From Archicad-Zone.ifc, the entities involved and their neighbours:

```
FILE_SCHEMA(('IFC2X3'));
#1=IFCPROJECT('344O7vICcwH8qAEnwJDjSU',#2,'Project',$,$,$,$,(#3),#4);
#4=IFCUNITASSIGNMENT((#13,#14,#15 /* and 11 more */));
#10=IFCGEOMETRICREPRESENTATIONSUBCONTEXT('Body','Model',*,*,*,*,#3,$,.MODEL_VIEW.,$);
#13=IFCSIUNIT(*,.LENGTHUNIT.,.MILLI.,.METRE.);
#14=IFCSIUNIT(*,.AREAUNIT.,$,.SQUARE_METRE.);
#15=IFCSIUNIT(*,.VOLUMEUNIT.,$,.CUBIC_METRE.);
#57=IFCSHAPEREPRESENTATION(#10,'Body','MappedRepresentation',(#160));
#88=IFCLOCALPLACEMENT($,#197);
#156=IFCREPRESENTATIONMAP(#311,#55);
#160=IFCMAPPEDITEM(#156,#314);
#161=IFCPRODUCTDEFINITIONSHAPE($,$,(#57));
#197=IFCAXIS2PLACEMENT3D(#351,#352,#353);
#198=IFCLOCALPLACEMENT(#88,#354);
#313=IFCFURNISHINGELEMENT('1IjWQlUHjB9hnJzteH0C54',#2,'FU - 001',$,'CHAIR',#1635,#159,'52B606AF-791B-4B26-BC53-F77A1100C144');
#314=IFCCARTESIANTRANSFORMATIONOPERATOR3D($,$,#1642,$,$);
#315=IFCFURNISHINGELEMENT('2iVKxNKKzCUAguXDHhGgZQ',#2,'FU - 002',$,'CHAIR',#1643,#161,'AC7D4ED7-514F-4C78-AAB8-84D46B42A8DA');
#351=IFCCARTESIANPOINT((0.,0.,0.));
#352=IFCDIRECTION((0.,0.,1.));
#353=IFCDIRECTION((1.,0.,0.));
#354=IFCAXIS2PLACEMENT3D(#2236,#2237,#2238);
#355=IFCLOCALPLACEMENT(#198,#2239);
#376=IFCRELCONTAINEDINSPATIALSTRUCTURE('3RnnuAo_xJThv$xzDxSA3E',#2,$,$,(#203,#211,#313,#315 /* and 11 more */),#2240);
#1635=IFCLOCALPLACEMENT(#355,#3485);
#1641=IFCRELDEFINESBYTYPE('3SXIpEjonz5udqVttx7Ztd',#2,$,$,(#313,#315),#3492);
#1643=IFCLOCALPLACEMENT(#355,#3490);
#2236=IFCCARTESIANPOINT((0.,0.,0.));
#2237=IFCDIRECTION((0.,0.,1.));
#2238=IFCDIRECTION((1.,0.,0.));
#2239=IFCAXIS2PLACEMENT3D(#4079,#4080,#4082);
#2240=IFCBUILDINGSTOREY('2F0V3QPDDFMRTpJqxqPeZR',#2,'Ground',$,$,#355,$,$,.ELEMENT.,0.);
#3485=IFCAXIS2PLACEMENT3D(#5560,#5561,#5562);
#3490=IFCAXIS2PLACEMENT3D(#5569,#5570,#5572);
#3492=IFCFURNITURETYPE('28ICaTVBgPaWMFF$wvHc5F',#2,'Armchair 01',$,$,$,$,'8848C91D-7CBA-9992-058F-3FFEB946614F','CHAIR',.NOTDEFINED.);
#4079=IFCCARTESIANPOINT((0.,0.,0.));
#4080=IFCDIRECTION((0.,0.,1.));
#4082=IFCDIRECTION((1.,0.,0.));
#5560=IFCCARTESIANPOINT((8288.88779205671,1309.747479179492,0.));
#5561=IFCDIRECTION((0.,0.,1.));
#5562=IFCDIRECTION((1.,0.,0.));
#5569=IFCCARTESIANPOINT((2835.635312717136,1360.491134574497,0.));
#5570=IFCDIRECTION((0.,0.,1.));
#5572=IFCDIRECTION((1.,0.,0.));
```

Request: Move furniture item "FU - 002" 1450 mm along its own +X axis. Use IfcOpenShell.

```python
import ifcopenshell
import ifcopenshell.api.geometry
import ifcopenshell.util.placement
import ifcopenshell.util.unit

model = ifcopenshell.open("Archicad-Zone.ifc")
unit_scale = ifcopenshell.util.unit.calculate_unit_scale(model)

item = model.by_guid("2iVKxNKKzCUAguXDHhGgZQ")
matrix = ifcopenshell.util.placement.get_local_placement(item.ObjectPlacement)
matrix[:3, 3] += matrix[:3, 0] * 1.45 / unit_scale
ifcopenshell.api.geometry.edit_object_placement(model, product=item, matrix=matrix, is_si=False)

print(ifcopenshell.util.placement.get_local_placement(item.ObjectPlacement).round(3) + 0.0)

model.write("Archicad-Zone-out.ifc")
```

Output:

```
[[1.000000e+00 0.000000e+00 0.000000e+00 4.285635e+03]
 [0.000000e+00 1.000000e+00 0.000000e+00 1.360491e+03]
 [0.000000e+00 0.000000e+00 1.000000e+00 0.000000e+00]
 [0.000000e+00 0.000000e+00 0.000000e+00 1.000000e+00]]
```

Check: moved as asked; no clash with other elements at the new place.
